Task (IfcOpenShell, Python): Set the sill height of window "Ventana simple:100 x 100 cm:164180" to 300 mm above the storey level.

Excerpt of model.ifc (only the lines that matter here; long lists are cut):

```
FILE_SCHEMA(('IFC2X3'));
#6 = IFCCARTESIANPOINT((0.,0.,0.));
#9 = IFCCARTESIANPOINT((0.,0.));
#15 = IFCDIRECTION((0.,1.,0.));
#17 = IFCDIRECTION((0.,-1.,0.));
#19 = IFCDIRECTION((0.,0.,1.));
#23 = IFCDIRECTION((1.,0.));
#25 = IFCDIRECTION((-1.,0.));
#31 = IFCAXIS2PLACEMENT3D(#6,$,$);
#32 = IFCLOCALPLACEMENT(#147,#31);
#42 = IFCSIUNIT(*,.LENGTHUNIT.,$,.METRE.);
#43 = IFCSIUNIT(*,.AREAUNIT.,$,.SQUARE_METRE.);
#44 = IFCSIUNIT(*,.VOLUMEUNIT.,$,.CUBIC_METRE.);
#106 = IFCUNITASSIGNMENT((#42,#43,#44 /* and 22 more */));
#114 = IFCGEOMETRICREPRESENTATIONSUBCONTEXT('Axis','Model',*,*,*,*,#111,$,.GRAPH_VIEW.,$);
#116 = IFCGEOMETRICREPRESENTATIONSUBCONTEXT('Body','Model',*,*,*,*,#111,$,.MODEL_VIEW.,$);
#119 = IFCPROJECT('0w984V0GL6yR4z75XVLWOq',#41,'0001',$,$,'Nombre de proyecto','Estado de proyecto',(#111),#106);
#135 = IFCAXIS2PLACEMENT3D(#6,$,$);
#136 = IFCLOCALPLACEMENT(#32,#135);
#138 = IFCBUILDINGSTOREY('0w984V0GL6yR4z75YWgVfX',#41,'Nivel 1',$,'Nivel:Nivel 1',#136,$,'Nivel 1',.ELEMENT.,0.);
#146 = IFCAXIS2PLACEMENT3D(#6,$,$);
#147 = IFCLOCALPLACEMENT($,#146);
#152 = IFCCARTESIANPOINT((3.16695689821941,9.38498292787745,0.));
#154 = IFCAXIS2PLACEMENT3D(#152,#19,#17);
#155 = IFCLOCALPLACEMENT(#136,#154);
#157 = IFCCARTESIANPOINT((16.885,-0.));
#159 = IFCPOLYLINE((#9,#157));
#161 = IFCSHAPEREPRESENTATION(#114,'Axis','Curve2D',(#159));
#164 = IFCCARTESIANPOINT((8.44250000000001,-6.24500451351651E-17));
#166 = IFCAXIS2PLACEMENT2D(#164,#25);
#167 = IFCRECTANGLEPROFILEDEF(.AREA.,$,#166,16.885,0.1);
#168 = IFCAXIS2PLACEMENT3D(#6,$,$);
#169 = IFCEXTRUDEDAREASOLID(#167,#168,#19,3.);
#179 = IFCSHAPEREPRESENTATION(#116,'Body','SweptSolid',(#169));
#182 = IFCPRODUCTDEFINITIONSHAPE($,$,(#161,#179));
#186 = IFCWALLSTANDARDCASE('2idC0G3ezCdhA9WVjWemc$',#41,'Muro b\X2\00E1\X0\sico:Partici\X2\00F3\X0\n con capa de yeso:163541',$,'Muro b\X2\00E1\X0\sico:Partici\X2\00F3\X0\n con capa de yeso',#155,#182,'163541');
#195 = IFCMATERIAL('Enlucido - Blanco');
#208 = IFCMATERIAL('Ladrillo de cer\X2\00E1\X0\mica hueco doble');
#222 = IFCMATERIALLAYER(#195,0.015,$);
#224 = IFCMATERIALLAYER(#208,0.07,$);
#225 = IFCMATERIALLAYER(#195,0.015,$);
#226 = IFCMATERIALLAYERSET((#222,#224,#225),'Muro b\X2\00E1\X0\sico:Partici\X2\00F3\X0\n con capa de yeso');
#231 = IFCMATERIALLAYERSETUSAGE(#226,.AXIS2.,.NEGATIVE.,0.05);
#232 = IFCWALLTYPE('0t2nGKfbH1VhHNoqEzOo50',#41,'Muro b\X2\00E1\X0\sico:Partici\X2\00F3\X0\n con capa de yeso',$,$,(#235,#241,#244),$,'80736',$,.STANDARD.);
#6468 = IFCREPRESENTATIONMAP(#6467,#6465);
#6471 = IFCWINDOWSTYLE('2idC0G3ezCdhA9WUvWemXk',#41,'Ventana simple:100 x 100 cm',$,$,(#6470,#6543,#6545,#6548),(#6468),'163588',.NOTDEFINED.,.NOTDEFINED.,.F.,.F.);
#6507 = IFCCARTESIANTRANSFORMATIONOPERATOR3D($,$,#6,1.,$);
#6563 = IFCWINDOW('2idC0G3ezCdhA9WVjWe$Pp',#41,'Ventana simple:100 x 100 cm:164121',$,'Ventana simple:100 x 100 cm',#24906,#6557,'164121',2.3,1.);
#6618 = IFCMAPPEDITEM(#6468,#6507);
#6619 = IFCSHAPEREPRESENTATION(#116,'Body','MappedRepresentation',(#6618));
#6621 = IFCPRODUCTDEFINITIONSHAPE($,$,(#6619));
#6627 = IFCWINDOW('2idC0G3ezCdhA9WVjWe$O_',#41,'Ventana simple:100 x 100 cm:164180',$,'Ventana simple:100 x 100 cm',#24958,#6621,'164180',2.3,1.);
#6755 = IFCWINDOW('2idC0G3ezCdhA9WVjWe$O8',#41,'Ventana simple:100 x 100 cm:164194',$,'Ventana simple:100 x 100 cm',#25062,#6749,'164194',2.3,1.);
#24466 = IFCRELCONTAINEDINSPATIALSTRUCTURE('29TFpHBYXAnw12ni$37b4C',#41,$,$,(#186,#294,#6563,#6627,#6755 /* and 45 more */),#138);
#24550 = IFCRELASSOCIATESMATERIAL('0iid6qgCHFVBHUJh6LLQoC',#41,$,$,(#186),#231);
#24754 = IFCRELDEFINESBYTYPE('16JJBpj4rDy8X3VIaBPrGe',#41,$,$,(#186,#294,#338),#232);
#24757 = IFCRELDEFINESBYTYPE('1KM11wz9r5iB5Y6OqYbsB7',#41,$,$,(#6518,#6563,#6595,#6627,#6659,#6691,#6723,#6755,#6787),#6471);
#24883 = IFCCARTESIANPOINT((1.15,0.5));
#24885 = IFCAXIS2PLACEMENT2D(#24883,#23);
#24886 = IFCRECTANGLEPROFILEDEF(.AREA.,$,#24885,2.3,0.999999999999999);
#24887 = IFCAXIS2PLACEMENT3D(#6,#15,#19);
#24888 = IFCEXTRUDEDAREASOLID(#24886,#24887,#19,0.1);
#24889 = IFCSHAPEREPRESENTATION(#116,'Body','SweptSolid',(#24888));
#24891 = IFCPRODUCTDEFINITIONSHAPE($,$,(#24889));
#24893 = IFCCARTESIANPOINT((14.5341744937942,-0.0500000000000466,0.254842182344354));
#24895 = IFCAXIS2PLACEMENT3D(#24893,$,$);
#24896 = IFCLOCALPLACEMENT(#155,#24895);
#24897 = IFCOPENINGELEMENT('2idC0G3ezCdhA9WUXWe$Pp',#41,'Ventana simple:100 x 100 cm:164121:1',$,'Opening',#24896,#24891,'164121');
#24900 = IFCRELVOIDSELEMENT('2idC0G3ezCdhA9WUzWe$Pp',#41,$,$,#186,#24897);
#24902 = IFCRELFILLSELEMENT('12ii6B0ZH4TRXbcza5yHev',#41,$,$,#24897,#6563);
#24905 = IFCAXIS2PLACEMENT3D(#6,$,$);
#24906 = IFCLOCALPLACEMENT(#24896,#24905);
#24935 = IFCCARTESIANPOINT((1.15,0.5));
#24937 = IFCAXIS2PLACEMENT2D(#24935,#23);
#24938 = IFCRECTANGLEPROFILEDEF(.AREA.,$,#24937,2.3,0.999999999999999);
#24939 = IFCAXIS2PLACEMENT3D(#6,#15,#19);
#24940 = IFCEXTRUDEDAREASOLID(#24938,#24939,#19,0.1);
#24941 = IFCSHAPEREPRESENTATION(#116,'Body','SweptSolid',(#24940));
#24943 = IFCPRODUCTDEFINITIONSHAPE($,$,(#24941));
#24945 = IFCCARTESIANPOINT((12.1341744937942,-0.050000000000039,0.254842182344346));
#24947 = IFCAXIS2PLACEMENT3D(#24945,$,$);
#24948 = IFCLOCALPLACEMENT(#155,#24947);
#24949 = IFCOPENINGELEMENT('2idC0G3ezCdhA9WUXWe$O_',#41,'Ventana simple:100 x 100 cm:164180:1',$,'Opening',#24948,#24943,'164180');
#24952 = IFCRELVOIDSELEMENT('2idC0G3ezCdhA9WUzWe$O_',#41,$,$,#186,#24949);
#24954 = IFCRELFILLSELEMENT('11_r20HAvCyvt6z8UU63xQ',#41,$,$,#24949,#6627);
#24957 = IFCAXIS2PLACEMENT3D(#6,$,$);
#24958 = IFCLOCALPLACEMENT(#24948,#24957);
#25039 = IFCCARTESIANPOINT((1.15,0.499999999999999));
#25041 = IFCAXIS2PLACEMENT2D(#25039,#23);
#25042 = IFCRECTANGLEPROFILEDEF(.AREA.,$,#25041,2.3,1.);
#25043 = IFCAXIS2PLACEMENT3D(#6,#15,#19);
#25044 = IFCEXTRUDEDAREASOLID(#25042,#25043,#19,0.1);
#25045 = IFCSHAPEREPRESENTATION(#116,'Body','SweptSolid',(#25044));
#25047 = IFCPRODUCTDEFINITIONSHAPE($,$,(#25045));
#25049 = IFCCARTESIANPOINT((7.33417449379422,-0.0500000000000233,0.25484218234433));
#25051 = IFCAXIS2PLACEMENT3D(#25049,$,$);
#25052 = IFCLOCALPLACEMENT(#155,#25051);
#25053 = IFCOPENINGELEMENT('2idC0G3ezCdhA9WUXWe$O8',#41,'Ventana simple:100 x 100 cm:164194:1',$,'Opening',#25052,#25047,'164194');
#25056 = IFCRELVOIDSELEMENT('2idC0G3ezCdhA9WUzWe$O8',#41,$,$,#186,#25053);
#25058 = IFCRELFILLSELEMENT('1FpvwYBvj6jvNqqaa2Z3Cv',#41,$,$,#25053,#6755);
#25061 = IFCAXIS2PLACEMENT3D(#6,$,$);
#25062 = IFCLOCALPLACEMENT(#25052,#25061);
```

```python
import numpy as np
import ifcopenshell
import ifcopenshell.api.geometry
import ifcopenshell.geom
import ifcopenshell.util.element
import ifcopenshell.util.placement
import ifcopenshell.util.shape
import ifcopenshell.util.unit

model = ifcopenshell.open("model.ifc")
unit_scale = ifcopenshell.util.unit.calculate_unit_scale(model)

window = model.by_guid("2idC0G3ezCdhA9WVjWe$O_")
opening = window.FillsVoids[0].RelatingOpeningElement
storey = ifcopenshell.util.element.get_container(window, ifc_class="IfcBuildingStorey")
level = ifcopenshell.util.placement.get_local_placement(storey.ObjectPlacement)[2, 3]

# The opening's origin need not be at the sill, so measure its lowest point.
shape = ifcopenshell.geom.create_shape(ifcopenshell.geom.settings(), opening)
bottom = ifcopenshell.util.shape.get_shape_bottom_elevation(shape, shape.geometry) / unit_scale
dz = level + 0.3 / unit_scale - bottom

shift = np.array([0.0, 0.0, dz])
# The window is placed relative to its opening, so it follows when the opening moves.
matrix = ifcopenshell.util.placement.get_local_placement(opening.ObjectPlacement)
matrix[:3, 3] += shift
ifcopenshell.api.geometry.edit_object_placement(
    model, product=opening, matrix=matrix, is_si=False, should_transform_children=True
)

print(f"moved by {dz * unit_scale:+.3f} m")

model.write("model_edited.ifc")
```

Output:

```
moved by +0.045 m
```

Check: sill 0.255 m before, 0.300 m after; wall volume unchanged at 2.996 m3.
